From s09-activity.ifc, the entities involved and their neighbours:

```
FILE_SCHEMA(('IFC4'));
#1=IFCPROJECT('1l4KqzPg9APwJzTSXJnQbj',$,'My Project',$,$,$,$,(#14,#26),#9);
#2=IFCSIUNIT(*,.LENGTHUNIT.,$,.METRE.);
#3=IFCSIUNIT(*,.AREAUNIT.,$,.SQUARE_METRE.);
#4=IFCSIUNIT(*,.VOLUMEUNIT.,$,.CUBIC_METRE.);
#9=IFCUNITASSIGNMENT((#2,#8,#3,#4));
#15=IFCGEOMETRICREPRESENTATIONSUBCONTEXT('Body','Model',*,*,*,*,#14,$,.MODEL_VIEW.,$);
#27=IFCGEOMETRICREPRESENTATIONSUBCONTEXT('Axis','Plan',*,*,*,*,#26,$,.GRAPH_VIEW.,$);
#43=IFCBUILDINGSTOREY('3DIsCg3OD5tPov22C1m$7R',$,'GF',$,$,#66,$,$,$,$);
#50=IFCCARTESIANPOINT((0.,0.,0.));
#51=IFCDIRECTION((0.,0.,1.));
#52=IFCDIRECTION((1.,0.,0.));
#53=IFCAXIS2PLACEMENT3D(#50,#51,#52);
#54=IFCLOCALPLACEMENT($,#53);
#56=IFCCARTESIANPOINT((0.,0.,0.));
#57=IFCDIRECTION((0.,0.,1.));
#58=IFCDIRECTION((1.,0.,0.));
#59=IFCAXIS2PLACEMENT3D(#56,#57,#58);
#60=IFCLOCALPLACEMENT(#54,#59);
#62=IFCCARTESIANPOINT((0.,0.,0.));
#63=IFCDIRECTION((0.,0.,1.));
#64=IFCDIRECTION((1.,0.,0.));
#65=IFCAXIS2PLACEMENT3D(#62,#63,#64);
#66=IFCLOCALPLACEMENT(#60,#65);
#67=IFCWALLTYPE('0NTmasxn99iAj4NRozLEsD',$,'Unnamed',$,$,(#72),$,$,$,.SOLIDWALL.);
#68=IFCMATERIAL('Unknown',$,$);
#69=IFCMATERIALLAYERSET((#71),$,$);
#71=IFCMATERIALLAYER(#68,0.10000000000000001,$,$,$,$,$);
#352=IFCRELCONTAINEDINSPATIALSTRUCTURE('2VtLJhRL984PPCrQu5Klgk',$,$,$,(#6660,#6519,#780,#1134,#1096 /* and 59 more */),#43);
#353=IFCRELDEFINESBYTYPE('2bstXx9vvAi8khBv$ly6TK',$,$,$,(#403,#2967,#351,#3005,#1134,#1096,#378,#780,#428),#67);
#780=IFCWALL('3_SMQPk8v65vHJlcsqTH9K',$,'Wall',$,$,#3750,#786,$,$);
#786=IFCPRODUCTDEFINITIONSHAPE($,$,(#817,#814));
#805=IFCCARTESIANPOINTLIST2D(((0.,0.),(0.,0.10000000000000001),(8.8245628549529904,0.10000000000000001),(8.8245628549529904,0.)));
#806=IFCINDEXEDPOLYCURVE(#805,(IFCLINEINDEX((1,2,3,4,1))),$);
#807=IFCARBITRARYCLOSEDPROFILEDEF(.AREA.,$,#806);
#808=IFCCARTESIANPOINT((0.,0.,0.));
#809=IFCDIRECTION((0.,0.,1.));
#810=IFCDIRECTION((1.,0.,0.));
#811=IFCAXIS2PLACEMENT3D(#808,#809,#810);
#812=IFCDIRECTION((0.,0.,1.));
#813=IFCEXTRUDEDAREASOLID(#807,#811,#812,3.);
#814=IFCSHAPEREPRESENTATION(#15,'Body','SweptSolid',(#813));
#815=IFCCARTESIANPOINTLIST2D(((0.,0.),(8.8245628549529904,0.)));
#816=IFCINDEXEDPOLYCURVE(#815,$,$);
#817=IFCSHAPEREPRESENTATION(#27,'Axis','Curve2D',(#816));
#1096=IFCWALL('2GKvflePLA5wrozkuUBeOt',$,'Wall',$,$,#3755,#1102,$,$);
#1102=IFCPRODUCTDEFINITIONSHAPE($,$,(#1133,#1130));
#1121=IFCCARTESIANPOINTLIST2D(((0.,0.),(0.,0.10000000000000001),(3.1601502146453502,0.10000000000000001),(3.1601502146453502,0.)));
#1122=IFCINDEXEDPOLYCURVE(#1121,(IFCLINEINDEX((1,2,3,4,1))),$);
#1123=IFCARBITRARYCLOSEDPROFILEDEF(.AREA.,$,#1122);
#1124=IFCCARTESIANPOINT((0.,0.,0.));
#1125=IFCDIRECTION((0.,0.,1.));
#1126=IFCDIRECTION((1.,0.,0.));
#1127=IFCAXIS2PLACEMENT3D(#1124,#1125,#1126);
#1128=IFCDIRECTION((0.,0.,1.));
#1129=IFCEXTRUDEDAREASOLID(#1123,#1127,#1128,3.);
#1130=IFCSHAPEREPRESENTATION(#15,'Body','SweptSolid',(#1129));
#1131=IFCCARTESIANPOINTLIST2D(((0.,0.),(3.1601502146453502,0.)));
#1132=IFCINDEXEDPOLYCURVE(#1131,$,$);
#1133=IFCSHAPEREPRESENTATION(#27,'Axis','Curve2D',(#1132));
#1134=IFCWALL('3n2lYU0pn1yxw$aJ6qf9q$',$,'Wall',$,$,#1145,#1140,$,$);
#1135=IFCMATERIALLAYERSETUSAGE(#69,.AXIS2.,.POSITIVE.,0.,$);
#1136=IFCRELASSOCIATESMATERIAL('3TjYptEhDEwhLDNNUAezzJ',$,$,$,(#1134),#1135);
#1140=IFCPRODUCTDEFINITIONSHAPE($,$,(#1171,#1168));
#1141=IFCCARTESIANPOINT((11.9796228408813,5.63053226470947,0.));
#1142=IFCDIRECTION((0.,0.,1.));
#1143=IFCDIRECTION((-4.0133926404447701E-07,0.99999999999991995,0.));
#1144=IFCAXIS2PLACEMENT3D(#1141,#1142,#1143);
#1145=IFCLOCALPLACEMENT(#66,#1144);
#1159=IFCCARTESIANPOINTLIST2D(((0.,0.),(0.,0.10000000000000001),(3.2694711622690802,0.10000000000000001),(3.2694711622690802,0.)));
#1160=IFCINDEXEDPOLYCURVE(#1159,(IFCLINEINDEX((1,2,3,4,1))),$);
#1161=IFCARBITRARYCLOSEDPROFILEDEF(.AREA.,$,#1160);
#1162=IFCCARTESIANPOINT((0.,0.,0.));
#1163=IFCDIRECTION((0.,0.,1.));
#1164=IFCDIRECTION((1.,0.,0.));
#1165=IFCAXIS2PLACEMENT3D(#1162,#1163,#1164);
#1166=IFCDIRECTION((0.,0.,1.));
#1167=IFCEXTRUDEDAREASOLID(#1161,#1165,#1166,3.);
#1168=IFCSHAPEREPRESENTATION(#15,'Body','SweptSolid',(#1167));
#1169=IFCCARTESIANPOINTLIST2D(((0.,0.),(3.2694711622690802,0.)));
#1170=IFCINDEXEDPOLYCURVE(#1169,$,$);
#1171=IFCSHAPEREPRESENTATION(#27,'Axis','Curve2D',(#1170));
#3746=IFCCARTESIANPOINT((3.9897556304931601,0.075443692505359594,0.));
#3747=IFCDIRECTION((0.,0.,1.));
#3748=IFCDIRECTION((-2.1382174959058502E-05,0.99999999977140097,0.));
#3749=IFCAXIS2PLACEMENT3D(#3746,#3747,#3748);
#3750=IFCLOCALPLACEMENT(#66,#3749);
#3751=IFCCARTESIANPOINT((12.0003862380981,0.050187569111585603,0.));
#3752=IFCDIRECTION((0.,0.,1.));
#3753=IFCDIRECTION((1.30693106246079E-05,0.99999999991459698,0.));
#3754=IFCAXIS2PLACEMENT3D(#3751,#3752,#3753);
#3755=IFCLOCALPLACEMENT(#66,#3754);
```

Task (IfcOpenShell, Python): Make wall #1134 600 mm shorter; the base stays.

```python
import ifcopenshell
import ifcopenshell.geom
import ifcopenshell.util.representation
import ifcopenshell.util.shape
import ifcopenshell.util.unit

model = ifcopenshell.open("s09-activity.ifc")
unit_scale = ifcopenshell.util.unit.calculate_unit_scale(model)
settings = ifcopenshell.geom.settings()


def volume(element):
    """Net volume in cubic metres, openings subtracted."""
    shape = ifcopenshell.geom.create_shape(settings, element)
    return ifcopenshell.util.shape.get_volume(shape.geometry)


wall = model.by_guid("3n2lYU0pn1yxw$aJ6qf9q$")
before = volume(wall)

body = ifcopenshell.util.representation.get_representation(wall, "Model", "Body")
solid = body.Items[0]
old_height = solid.Depth
solid.Depth -= 0.6 / unit_scale
after = volume(wall)

print(f"height {old_height:g} -> {solid.Depth:g}, volume {before:.3f} -> {after:.3f} m3")

model.write("s09-activity_rev.ifc")
```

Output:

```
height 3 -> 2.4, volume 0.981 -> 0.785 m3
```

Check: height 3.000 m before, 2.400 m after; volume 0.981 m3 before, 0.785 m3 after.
